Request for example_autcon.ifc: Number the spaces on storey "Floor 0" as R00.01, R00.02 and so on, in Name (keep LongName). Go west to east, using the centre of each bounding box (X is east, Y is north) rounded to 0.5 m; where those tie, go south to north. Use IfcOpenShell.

First a look at what the model holds.

```python
import ifcopenshell
import ifcopenshell.util.element
import ifcopenshell.util.placement

model = ifcopenshell.open("example_autcon.ifc")
print(model.schema)
storey = next(s for s in model.by_type("IfcBuildingStorey") if s.Name == "Floor 0")
spaces = [e for e in ifcopenshell.util.element.get_decomposition(storey) if e.is_a("IfcSpace")]
for e in sorted(spaces, key=lambda e: e.id()):
    origin = ifcopenshell.util.placement.get_local_placement(e.ObjectPlacement)[:3, 3]
    print(e.id(), e.Name, e.LongName, origin.round(2) + 0.0, sep=" | ")
```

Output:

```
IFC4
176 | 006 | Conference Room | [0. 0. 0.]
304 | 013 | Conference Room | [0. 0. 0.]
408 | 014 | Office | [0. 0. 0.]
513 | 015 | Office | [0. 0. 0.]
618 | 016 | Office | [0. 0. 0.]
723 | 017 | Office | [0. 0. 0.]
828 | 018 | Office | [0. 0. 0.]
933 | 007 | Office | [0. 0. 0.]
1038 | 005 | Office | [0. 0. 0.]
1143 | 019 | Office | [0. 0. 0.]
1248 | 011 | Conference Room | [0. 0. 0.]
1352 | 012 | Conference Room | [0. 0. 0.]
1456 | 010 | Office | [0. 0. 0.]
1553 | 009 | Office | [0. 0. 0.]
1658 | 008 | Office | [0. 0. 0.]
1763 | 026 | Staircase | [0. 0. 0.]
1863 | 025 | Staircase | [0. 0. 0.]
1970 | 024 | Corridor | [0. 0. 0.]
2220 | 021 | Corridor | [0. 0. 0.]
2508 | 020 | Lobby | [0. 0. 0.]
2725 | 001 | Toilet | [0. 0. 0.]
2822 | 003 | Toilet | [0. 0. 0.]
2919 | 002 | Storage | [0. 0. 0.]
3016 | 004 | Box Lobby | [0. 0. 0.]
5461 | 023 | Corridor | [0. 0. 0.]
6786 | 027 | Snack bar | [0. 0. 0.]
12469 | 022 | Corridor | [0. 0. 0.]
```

```python
import ifcopenshell
import ifcopenshell.geom
import ifcopenshell.util.element
import ifcopenshell.util.shape

model = ifcopenshell.open("example_autcon.ifc")
settings = ifcopenshell.geom.settings()
settings.set("use-world-coords", True)


def centre(element):
    shape = ifcopenshell.geom.create_shape(settings, element)
    return ifcopenshell.util.shape.get_bbox_centroid(shape.geometry)


storey = next(s for s in model.by_type("IfcBuildingStorey") if s.Name == "Floor 0")
spaces = [e for e in ifcopenshell.util.element.get_decomposition(storey) if e.is_a("IfcSpace")]

# Insertion points can sit at a corner or the storey origin, so sort by the geometry (in metres).
centres = {e: centre(e) for e in spaces}
spaces.sort(key=lambda e: (round(centres[e][0] / 0.5), centres[e][1]))

for i, e in enumerate(spaces, start=1):
    number = f"R00.{i:02d}"
    e.Name = number
    print(e.id(), number)

model.write("example_autcon_v2.ifc")
```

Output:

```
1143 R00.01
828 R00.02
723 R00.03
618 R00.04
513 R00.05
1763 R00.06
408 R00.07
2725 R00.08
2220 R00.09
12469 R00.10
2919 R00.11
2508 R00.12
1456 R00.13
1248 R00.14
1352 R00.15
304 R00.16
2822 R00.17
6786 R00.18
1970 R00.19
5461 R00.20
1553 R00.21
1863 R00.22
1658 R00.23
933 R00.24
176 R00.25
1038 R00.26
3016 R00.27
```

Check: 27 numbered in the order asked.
